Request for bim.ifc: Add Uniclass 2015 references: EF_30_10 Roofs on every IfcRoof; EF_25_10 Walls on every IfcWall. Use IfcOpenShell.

First a look at what the model holds.

```python
import ifcopenshell

model = ifcopenshell.open("bim.ifc")
print(model.schema)
print("classifications:", [c.Name for c in model.by_type("IfcClassification")])
for ifc_class in ("IfcDoor", "IfcRoof", "IfcStair", "IfcWall", "IfcWindow"):
    print(ifc_class, len(model.by_type(ifc_class)))
```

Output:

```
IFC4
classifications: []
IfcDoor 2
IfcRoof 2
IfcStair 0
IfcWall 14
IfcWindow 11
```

```python
import ifcopenshell
import ifcopenshell.api.classification

model = ifcopenshell.open("bim.ifc")

system = ifcopenshell.api.classification.add_classification(model, classification="Uniclass 2015")

codes = {
    "IfcRoof": ("EF_30_10", "Roofs"),
    "IfcWall": ("EF_25_10", "Walls"),
}
for ifc_class, (code, name) in codes.items():
    products = model.by_type(ifc_class)
    ifcopenshell.api.classification.add_reference(
        model, products=products, classification=system, identification=code, name=name
    )
    print(code, len(products))

model.write("bim_v2.ifc")
```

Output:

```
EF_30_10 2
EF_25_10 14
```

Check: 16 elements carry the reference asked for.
